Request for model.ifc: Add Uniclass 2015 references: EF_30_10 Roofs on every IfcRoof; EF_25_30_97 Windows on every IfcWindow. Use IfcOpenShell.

First a look at what the model holds.

```python
import ifcopenshell

model = ifcopenshell.open("model.ifc")
print(model.schema)
print("classifications:", [c.Name for c in model.by_type("IfcClassification")])
for ifc_class in ("IfcDoor", "IfcRoof", "IfcStair", "IfcWall", "IfcWindow"):
    print(ifc_class, len(model.by_type(ifc_class)))
```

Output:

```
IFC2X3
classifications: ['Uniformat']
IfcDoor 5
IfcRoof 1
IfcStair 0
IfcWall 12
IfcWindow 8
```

```python
import ifcopenshell
import ifcopenshell.api.classification

model = ifcopenshell.open("model.ifc")

# IFC2X3 requires Source and Edition and has no link from the project to the system.
system = model.create_entity("IfcClassification", Source="NBS", Edition="2015", Name="Uniclass 2015")

codes = {
    "IfcRoof": ("EF_30_10", "Roofs"),
    "IfcWindow": ("EF_25_30_97", "Windows"),
}
for ifc_class, (code, name) in codes.items():
    products = model.by_type(ifc_class)
    ifcopenshell.api.classification.add_reference(
        model, products=products, classification=system, identification=code, name=name
    )
    print(code, len(products))

model.write("model_updated.ifc")
```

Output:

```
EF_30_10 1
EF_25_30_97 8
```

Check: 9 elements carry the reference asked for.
